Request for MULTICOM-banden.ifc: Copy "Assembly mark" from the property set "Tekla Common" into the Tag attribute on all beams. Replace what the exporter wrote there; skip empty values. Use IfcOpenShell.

First a look at what the model holds.

```python
import ifcopenshell
import ifcopenshell.util.element

model = ifcopenshell.open("MULTICOM-banden.ifc")
print(model.schema)
beams = model.by_type("IfcBeam")
print(len(beams), "beams")
for e in beams[:8]:
    source = ifcopenshell.util.element.get_pset(e, "Tekla Common", "Assembly mark")
    target = e.Tag
    print(e.id(), repr(source), repr(target), sep=" | ")
```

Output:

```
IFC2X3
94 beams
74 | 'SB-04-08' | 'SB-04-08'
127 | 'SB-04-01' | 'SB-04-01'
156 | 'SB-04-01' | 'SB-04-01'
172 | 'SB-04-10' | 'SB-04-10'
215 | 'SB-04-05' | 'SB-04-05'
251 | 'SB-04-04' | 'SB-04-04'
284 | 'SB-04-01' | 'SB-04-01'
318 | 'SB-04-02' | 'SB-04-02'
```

```python
import ifcopenshell
import ifcopenshell.util.element

model = ifcopenshell.open("MULTICOM-banden.ifc")

count = 0
for e in model.by_type("IfcBeam"):
    value = ifcopenshell.util.element.get_pset(e, "Tekla Common", "Assembly mark")
    current = e.Tag
    if not value or not value.strip() or current == value:
        continue
    e.Tag = value
    count += 1

print(count, "beams updated")

model.write("MULTICOM-banden_v2.ifc")
```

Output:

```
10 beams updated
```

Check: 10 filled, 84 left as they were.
